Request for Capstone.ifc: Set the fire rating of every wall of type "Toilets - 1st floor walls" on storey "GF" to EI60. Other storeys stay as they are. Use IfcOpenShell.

First a look at what the model holds.

```python
import ifcopenshell
import ifcopenshell.util.element

model = ifcopenshell.open("Capstone.ifc")
print(model.schema)
storey = next(s for s in model.by_type("IfcBuildingStorey") if s.Name == "GF")
walls = [e for e in ifcopenshell.util.element.get_decomposition(storey) if e.is_a("IfcWall")]
seen = {}
for e in walls:
    element_type = ifcopenshell.util.element.get_type(e)
    key = (element_type.Name if element_type != e and element_type else None, ifcopenshell.util.element.get_pset(e, "Pset_WallCommon", "FireRating"))
    seen[key] = seen.get(key, 0) + 1
for (name, value), count in sorted(seen.items(), key=str):
    print(count, "x", name, "|", value)
```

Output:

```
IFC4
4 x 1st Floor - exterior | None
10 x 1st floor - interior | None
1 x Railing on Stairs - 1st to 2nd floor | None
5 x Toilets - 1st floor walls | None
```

```python
import ifcopenshell
import ifcopenshell.api.pset
import ifcopenshell.util.element

model = ifcopenshell.open("Capstone.ifc")

storey = next(s for s in model.by_type("IfcBuildingStorey") if s.Name == "GF")
walls = [e for e in ifcopenshell.util.element.get_decomposition(storey) if e.is_a("IfcWall")]

count = 0
for e in walls:
    element_type = ifcopenshell.util.element.get_type(e)
    if element_type in (None, e) or element_type.Name != "Toilets - 1st floor walls":
        continue
    # add_pset returns the element's existing set when there is one.
    pset = ifcopenshell.api.pset.add_pset(model, product=e, name="Pset_WallCommon")
    ifcopenshell.api.pset.edit_pset(model, pset=pset, properties={"FireRating": "EI60"})
    count += 1

print(count, "walls updated")

model.write("Capstone_updated.ifc")
```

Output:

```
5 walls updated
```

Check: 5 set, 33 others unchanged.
